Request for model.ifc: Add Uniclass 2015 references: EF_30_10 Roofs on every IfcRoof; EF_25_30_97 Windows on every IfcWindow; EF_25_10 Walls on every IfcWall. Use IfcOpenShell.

First a look at what the model holds.

```python
import ifcopenshell

model = ifcopenshell.open("model.ifc")
print(model.schema)
print("classifications:", [c.Name for c in model.by_type("IfcClassification")])
for ifc_class in ("IfcDoor", "IfcRoof", "IfcStair", "IfcWall", "IfcWindow"):
    print(ifc_class, len(model.by_type(ifc_class)))
```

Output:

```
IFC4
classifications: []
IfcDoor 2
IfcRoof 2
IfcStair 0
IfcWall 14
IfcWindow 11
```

```python
import ifcopenshell
import ifcopenshell.api.classification

model = ifcopenshell.open("model.ifc")

system = ifcopenshell.api.classification.add_classification(model, classification="Uniclass 2015")

codes = {
    "IfcRoof": ("EF_30_10", "Roofs"),
    "IfcWindow": ("EF_25_30_97", "Windows"),
    "IfcWall": ("EF_25_10", "Walls"),
}
for ifc_class, (code, name) in codes.items():
    products = model.by_type(ifc_class)
    ifcopenshell.api.classification.add_reference(
        model, products=products, classification=system, identification=code, name=name
    )
    print(code, len(products))

model.write("model_updated.ifc")
```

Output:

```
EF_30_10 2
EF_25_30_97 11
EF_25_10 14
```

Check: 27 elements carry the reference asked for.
